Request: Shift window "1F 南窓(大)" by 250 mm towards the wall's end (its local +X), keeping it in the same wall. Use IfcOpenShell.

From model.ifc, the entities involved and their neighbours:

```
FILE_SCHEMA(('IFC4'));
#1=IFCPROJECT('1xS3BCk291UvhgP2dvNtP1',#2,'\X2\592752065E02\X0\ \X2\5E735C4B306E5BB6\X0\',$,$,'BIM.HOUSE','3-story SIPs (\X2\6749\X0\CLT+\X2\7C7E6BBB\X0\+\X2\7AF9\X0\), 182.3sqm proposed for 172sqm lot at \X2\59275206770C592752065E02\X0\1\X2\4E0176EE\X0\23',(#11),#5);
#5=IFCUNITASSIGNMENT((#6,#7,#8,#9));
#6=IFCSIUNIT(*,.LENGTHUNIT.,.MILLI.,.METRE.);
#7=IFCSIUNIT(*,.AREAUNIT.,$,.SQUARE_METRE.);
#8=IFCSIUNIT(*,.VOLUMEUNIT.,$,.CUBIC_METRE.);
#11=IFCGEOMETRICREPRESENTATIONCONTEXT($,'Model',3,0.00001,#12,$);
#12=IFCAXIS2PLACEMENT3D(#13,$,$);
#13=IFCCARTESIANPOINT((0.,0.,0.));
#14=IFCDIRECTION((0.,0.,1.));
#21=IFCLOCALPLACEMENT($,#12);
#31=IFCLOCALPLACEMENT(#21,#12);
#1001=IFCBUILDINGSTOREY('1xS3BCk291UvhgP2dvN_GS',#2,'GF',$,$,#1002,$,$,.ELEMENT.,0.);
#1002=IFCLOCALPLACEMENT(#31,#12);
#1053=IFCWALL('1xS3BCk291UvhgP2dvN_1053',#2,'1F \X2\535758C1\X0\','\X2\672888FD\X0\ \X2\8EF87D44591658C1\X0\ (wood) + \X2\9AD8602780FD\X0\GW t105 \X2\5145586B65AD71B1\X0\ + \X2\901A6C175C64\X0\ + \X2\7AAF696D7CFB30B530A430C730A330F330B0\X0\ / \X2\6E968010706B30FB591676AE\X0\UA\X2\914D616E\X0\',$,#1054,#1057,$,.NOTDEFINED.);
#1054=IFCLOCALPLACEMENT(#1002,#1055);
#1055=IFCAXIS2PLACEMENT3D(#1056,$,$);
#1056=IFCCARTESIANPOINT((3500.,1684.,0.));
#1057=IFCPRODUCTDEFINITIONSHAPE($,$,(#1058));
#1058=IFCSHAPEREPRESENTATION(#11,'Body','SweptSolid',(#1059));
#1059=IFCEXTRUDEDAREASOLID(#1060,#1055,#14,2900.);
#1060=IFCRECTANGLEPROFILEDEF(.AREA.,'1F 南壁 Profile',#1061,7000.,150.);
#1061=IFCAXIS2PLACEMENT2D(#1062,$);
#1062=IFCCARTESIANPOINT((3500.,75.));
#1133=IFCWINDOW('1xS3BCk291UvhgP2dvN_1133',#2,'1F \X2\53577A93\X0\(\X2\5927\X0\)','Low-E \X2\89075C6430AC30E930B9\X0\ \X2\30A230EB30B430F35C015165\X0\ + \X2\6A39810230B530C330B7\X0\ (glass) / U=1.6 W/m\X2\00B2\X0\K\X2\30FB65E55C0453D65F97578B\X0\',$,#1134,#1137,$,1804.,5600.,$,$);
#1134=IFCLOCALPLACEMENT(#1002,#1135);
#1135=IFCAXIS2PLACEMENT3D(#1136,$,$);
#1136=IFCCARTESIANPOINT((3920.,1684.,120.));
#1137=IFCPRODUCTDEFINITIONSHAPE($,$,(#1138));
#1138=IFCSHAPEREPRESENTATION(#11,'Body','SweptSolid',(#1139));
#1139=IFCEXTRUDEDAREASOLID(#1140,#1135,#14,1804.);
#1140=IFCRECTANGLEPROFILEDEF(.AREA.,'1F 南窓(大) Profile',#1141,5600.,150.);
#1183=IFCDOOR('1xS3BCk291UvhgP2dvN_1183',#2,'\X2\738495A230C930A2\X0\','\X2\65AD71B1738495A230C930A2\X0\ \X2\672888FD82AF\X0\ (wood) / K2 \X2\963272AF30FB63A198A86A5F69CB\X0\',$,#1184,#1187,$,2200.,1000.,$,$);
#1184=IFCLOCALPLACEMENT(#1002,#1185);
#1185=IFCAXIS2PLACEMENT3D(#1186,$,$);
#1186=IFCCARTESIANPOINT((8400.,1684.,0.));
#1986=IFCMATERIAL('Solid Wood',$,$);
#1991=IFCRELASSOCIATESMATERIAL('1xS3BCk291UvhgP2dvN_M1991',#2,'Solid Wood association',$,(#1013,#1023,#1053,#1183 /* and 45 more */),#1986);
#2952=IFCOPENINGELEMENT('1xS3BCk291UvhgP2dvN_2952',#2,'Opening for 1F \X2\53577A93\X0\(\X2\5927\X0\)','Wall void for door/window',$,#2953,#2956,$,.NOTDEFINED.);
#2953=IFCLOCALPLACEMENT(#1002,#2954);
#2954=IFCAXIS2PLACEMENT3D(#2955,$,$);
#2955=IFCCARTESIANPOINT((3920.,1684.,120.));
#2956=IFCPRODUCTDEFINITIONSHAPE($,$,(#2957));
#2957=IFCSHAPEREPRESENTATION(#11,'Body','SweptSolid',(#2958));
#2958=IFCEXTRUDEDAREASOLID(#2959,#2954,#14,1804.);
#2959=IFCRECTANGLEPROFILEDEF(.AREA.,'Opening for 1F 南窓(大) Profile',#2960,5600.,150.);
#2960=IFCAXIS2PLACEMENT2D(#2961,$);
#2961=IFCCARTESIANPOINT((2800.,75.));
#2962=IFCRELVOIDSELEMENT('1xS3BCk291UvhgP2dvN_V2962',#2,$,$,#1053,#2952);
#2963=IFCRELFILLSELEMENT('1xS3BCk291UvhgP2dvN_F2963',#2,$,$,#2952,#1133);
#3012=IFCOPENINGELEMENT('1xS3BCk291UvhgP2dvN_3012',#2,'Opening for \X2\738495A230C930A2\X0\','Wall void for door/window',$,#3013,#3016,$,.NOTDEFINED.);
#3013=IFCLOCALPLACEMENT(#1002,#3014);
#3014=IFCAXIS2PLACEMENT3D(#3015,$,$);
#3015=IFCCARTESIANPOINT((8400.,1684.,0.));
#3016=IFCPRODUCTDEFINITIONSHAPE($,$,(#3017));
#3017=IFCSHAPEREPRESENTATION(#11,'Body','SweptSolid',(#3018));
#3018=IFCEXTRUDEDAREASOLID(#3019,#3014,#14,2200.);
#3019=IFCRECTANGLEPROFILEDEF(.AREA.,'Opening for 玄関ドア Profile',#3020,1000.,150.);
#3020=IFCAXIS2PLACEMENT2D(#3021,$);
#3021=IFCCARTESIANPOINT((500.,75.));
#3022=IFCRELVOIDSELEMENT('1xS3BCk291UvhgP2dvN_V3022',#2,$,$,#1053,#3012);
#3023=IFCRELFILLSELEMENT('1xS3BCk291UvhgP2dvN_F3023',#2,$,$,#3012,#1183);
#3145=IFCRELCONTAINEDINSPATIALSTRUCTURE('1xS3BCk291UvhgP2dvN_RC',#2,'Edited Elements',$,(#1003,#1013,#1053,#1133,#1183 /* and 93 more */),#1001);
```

```python
import ifcopenshell
import ifcopenshell.api.geometry
import ifcopenshell.util.placement
import ifcopenshell.util.unit

model = ifcopenshell.open("model.ifc")
unit_scale = ifcopenshell.util.unit.calculate_unit_scale(model)

window = model.by_guid("1xS3BCk291UvhgP2dvN_1133")
opening = window.FillsVoids[0].RelatingOpeningElement
wall = opening.VoidsElements[0].RelatingBuildingElement

wall_matrix = ifcopenshell.util.placement.get_local_placement(wall.ObjectPlacement)
shift = wall_matrix[:3, 0] * 0.25 / unit_scale
before = ifcopenshell.util.placement.get_local_placement(window.ObjectPlacement)[:3, 3].copy()

# The window is not placed relative to its opening, so move both.
for product in (opening, window):
    matrix = ifcopenshell.util.placement.get_local_placement(product.ObjectPlacement)
    matrix[:3, 3] += shift
    ifcopenshell.api.geometry.edit_object_placement(model, product=product, matrix=matrix, is_si=False)

after = ifcopenshell.util.placement.get_local_placement(window.ObjectPlacement)[:3, 3]
print("window moved by", (after - before).round(3) + 0.0)

model.write("model_updated.ifc")
```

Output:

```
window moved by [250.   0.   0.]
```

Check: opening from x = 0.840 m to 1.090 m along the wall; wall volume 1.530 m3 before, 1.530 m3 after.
